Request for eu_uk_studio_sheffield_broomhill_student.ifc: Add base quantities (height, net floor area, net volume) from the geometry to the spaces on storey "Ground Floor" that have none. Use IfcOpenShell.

First a look at what the model holds.

```python
import ifcopenshell
import ifcopenshell.util.element
import ifcopenshell.util.unit

model = ifcopenshell.open("eu_uk_studio_sheffield_broomhill_student.ifc")
print(model.schema)
for unit_type in ("LENGTHUNIT", "AREAUNIT", "VOLUMEUNIT"):
    print(unit_type, ifcopenshell.util.unit.calculate_unit_scale(model, unit_type))
storey = next(s for s in model.by_type("IfcBuildingStorey") if s.Name == "Ground Floor")
spaces = [e for e in ifcopenshell.util.element.get_decomposition(storey) if e.is_a("IfcSpace")]
for e in sorted(spaces, key=lambda e: e.id()):
    print(e.id(), e.is_a(), e.Name, list(ifcopenshell.util.element.get_psets(e, qtos_only=True)), sep=" | ")
```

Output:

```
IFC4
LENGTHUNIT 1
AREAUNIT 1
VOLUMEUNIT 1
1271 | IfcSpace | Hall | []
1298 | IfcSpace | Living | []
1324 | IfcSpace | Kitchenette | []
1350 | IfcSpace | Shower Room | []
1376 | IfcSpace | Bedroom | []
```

```python
import ifcopenshell
import ifcopenshell.api.pset
import ifcopenshell.geom
import ifcopenshell.util.element
import ifcopenshell.util.shape
import ifcopenshell.util.unit

model = ifcopenshell.open("eu_uk_studio_sheffield_broomhill_student.ifc")
unit_scale = ifcopenshell.util.unit.calculate_unit_scale(model)
area_scale = ifcopenshell.util.unit.calculate_unit_scale(model, "AREAUNIT")
volume_scale = ifcopenshell.util.unit.calculate_unit_scale(model, "VOLUMEUNIT")
settings = ifcopenshell.geom.settings()

storey = next(s for s in model.by_type("IfcBuildingStorey") if s.Name == "Ground Floor")
spaces = [e for e in ifcopenshell.util.element.get_decomposition(storey) if e.is_a("IfcSpace")]

for e in sorted(spaces, key=lambda e: e.id()):
    if ifcopenshell.util.element.get_psets(e, qtos_only=True, should_inherit=False):
        continue
    # Geometry comes back in metres, in the element's own axes.
    shape = ifcopenshell.geom.create_shape(settings, e)
    values = {
        "Height": ifcopenshell.util.shape.get_z(shape.geometry) / unit_scale,
        "NetFloorArea": ifcopenshell.util.shape.get_footprint_area(shape.geometry) / area_scale,
        "NetVolume": ifcopenshell.util.shape.get_volume(shape.geometry) / volume_scale,
    }
    qto = ifcopenshell.api.pset.add_qto(model, product=e, name="Qto_SpaceBaseQuantities")
    ifcopenshell.api.pset.edit_qto(model, qto=qto, properties=values)
    print(e.id(), {k: round(v, 3) for k, v in values.items()})

model.write("eu_uk_studio_sheffield_broomhill_student-out.ifc")
```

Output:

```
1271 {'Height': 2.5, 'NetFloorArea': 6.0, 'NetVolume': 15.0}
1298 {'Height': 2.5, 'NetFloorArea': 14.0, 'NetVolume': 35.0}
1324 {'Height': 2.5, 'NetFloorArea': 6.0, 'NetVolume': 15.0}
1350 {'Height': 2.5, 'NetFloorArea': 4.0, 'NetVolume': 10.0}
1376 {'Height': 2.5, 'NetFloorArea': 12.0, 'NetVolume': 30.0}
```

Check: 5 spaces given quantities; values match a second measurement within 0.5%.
